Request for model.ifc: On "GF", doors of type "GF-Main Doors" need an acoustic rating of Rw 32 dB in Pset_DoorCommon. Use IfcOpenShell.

First a look at what the model holds.

```python
import ifcopenshell
import ifcopenshell.util.element

model = ifcopenshell.open("model.ifc")
print(model.schema)
storey = next(s for s in model.by_type("IfcBuildingStorey") if s.Name == "GF")
doors = [e for e in ifcopenshell.util.element.get_decomposition(storey) if e.is_a("IfcDoor")]
seen = {}
for e in doors:
    element_type = ifcopenshell.util.element.get_type(e)
    key = (element_type.Name if element_type != e and element_type else None, ifcopenshell.util.element.get_pset(e, "Pset_DoorCommon", "AcousticRating"))
    seen[key] = seen.get(key, 0) + 1
for (name, value), count in sorted(seen.items(), key=str):
    print(count, "x", name, "|", value)
```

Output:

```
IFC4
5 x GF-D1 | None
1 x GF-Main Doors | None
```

```python
import ifcopenshell
import ifcopenshell.api.pset
import ifcopenshell.util.element

model = ifcopenshell.open("model.ifc")

storey = next(s for s in model.by_type("IfcBuildingStorey") if s.Name == "GF")
doors = [e for e in ifcopenshell.util.element.get_decomposition(storey) if e.is_a("IfcDoor")]

count = 0
for e in doors:
    element_type = ifcopenshell.util.element.get_type(e)
    if element_type in (None, e) or element_type.Name != "GF-Main Doors":
        continue
    # add_pset returns the element's existing set when there is one.
    pset = ifcopenshell.api.pset.add_pset(model, product=e, name="Pset_DoorCommon")
    ifcopenshell.api.pset.edit_pset(model, pset=pset, properties={"AcousticRating": "Rw 32 dB"})
    count += 1

print(count, "doors updated")

model.write("model_rev.ifc")
```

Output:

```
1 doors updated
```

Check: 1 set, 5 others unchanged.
